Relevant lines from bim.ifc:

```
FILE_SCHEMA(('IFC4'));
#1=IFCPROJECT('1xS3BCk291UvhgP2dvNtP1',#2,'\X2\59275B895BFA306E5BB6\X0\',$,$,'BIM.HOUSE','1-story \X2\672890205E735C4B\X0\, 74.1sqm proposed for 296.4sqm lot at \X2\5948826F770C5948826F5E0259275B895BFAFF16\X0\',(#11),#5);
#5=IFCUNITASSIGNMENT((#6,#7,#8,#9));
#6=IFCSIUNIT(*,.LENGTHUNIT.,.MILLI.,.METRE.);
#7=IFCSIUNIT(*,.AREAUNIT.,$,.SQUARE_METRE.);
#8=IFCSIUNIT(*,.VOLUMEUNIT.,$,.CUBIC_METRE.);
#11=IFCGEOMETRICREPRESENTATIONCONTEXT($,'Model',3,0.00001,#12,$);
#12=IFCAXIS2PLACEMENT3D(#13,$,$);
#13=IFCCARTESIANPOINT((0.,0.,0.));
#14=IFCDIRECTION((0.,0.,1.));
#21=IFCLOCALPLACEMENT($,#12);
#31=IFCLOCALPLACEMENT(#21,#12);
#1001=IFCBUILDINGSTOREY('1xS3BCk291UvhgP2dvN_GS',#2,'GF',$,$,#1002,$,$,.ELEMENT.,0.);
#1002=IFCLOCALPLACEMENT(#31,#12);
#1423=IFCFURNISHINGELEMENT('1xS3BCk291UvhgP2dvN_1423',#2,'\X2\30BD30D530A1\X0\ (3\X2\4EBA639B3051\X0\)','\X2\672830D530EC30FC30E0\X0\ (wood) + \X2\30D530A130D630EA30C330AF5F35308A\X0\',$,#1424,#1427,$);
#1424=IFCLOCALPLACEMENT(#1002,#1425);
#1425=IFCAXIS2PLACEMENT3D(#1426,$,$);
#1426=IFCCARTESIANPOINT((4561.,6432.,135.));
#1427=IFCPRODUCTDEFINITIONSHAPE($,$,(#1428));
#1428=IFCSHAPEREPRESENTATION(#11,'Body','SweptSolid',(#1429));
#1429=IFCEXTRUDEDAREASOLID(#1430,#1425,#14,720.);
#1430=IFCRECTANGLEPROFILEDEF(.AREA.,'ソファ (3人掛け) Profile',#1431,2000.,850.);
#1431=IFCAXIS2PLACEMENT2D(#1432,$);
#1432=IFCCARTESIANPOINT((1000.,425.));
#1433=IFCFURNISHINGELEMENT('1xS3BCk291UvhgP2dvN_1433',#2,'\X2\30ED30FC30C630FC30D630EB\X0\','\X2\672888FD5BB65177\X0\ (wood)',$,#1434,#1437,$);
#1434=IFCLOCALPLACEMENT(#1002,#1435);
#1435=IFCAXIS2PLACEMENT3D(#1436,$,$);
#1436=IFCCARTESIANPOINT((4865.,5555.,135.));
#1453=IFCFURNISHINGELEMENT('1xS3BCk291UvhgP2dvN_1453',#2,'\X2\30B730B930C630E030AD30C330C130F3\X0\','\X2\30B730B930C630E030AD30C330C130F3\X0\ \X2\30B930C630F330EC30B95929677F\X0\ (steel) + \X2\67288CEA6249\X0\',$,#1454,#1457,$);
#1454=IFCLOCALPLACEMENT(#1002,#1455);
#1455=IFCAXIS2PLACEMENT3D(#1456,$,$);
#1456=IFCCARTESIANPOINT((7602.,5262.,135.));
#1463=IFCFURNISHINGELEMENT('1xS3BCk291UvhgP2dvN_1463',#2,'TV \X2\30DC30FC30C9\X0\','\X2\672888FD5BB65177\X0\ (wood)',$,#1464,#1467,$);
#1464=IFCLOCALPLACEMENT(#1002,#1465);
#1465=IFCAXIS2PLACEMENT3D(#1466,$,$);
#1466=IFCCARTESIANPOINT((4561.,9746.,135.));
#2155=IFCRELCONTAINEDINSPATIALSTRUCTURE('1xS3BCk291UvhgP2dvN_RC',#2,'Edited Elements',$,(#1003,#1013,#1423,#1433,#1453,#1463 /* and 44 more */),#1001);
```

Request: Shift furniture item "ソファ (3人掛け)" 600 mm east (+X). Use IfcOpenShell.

```python
import ifcopenshell
import ifcopenshell.api.geometry
import ifcopenshell.util.placement

model = ifcopenshell.open("bim.ifc")

item = model.by_guid("1xS3BCk291UvhgP2dvN_1423")
matrix = ifcopenshell.util.placement.get_local_placement(item.ObjectPlacement)
matrix[0, 3] += 600.0
ifcopenshell.api.geometry.edit_object_placement(model, product=item, matrix=matrix, is_si=False)

print(ifcopenshell.util.placement.get_local_placement(item.ObjectPlacement).round(3) + 0.0)

model.write("bim-out.ifc")
```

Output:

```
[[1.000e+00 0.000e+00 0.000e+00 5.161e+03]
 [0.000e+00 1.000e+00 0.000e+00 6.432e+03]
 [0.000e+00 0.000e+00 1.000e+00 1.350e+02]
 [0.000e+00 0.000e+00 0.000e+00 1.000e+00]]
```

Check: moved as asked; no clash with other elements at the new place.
